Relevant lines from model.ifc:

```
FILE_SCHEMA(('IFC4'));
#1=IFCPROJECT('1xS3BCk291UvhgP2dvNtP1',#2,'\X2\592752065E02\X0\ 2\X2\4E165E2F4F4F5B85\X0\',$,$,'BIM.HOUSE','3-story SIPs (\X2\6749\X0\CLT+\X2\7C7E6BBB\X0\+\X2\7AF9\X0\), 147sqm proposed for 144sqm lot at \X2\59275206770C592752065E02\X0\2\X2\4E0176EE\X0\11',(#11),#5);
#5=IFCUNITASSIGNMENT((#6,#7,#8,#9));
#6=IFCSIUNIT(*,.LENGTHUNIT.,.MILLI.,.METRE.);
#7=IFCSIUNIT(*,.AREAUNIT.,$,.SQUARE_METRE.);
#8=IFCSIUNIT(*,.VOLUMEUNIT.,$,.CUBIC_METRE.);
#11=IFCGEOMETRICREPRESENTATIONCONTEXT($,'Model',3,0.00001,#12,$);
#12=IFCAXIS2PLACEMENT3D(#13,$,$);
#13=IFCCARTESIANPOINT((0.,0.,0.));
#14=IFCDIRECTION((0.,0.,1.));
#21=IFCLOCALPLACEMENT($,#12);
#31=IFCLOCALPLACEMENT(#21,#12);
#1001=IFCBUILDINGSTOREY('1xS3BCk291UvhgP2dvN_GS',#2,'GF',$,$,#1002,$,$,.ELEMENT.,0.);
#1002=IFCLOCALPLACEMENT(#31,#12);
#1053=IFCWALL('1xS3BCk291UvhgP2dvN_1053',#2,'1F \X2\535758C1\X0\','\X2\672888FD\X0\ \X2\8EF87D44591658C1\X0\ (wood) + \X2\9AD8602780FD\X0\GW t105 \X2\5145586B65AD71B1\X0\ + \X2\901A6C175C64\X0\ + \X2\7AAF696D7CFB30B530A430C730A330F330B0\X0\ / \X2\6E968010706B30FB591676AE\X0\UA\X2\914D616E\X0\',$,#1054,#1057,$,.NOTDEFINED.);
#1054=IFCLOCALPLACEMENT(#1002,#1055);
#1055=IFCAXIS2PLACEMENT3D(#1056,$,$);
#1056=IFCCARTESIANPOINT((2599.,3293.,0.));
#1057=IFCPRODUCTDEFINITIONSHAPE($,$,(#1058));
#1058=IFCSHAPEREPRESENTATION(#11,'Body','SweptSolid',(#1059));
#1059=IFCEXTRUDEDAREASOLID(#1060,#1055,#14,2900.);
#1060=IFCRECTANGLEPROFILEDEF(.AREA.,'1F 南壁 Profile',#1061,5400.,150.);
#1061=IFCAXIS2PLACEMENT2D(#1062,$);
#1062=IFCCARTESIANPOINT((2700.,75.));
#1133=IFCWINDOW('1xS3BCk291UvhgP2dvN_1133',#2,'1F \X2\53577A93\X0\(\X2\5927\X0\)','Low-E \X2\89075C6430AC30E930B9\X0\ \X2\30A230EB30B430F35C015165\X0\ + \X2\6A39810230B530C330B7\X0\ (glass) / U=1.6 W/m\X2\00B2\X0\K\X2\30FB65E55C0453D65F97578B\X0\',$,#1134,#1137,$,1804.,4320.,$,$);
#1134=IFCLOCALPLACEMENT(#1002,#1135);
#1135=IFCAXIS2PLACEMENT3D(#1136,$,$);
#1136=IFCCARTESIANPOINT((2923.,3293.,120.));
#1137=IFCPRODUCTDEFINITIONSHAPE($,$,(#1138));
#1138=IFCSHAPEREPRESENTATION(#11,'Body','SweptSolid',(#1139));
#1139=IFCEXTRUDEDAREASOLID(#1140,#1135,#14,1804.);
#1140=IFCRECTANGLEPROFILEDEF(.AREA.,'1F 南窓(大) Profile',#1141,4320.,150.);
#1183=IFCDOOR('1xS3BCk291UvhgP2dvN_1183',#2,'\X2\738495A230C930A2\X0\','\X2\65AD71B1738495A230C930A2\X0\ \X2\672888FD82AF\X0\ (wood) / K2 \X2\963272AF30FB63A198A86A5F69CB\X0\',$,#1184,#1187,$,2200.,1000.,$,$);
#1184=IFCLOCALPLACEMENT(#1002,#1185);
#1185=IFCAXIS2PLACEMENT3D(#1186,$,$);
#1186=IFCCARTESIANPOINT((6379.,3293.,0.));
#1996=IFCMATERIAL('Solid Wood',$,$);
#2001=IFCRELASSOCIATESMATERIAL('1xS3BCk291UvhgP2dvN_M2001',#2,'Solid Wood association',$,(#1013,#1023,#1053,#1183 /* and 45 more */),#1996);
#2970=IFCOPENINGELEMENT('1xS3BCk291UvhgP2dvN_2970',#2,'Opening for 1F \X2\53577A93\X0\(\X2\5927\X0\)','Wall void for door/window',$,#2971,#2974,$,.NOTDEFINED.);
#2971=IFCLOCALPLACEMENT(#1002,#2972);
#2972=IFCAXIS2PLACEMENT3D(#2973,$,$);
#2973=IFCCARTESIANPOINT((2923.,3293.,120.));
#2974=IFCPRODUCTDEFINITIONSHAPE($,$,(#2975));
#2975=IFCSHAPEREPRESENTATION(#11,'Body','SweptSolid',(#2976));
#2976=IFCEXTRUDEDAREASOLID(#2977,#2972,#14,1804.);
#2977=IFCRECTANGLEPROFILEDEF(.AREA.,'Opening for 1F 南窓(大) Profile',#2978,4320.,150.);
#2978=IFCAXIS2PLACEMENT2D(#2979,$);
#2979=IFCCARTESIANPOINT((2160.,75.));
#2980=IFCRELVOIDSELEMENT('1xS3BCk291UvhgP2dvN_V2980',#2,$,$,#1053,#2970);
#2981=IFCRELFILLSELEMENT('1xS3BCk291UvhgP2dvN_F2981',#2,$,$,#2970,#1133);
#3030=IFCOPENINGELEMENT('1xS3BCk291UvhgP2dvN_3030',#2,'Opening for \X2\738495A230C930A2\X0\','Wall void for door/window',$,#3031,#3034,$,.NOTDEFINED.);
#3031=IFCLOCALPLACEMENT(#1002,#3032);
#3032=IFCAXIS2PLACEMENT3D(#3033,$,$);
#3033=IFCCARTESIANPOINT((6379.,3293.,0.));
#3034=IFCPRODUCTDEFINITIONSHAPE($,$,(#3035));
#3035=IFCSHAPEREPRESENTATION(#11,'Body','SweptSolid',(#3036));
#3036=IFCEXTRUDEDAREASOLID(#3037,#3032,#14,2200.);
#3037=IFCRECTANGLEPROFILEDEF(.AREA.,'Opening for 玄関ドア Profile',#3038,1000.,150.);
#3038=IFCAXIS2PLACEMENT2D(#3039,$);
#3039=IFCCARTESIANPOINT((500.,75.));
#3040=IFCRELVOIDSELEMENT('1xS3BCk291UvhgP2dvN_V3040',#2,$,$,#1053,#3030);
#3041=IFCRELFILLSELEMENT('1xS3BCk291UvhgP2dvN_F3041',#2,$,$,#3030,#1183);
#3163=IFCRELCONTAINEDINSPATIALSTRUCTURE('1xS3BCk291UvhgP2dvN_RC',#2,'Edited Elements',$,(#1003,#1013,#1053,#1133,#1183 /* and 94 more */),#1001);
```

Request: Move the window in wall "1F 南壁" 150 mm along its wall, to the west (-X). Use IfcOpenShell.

```python
import ifcopenshell
import ifcopenshell.api.geometry
import ifcopenshell.util.placement
import ifcopenshell.util.unit

model = ifcopenshell.open("model.ifc")
unit_scale = ifcopenshell.util.unit.calculate_unit_scale(model)

window = model.by_guid("1xS3BCk291UvhgP2dvN_1133")
opening = window.FillsVoids[0].RelatingOpeningElement
wall = opening.VoidsElements[0].RelatingBuildingElement

wall_matrix = ifcopenshell.util.placement.get_local_placement(wall.ObjectPlacement)
shift = wall_matrix[:3, 0] * -0.15 / unit_scale
before = ifcopenshell.util.placement.get_local_placement(window.ObjectPlacement)[:3, 3].copy()

# The window is not placed relative to its opening, so move both.
for product in (opening, window):
    matrix = ifcopenshell.util.placement.get_local_placement(product.ObjectPlacement)
    matrix[:3, 3] += shift
    ifcopenshell.api.geometry.edit_object_placement(model, product=product, matrix=matrix, is_si=False)

after = ifcopenshell.util.placement.get_local_placement(window.ObjectPlacement)[:3, 3]
print("window moved by", (after - before).round(3) + 0.0)

model.write("model_edited.ifc")
```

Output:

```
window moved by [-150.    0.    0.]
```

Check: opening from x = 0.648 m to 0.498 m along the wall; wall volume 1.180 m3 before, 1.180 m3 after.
